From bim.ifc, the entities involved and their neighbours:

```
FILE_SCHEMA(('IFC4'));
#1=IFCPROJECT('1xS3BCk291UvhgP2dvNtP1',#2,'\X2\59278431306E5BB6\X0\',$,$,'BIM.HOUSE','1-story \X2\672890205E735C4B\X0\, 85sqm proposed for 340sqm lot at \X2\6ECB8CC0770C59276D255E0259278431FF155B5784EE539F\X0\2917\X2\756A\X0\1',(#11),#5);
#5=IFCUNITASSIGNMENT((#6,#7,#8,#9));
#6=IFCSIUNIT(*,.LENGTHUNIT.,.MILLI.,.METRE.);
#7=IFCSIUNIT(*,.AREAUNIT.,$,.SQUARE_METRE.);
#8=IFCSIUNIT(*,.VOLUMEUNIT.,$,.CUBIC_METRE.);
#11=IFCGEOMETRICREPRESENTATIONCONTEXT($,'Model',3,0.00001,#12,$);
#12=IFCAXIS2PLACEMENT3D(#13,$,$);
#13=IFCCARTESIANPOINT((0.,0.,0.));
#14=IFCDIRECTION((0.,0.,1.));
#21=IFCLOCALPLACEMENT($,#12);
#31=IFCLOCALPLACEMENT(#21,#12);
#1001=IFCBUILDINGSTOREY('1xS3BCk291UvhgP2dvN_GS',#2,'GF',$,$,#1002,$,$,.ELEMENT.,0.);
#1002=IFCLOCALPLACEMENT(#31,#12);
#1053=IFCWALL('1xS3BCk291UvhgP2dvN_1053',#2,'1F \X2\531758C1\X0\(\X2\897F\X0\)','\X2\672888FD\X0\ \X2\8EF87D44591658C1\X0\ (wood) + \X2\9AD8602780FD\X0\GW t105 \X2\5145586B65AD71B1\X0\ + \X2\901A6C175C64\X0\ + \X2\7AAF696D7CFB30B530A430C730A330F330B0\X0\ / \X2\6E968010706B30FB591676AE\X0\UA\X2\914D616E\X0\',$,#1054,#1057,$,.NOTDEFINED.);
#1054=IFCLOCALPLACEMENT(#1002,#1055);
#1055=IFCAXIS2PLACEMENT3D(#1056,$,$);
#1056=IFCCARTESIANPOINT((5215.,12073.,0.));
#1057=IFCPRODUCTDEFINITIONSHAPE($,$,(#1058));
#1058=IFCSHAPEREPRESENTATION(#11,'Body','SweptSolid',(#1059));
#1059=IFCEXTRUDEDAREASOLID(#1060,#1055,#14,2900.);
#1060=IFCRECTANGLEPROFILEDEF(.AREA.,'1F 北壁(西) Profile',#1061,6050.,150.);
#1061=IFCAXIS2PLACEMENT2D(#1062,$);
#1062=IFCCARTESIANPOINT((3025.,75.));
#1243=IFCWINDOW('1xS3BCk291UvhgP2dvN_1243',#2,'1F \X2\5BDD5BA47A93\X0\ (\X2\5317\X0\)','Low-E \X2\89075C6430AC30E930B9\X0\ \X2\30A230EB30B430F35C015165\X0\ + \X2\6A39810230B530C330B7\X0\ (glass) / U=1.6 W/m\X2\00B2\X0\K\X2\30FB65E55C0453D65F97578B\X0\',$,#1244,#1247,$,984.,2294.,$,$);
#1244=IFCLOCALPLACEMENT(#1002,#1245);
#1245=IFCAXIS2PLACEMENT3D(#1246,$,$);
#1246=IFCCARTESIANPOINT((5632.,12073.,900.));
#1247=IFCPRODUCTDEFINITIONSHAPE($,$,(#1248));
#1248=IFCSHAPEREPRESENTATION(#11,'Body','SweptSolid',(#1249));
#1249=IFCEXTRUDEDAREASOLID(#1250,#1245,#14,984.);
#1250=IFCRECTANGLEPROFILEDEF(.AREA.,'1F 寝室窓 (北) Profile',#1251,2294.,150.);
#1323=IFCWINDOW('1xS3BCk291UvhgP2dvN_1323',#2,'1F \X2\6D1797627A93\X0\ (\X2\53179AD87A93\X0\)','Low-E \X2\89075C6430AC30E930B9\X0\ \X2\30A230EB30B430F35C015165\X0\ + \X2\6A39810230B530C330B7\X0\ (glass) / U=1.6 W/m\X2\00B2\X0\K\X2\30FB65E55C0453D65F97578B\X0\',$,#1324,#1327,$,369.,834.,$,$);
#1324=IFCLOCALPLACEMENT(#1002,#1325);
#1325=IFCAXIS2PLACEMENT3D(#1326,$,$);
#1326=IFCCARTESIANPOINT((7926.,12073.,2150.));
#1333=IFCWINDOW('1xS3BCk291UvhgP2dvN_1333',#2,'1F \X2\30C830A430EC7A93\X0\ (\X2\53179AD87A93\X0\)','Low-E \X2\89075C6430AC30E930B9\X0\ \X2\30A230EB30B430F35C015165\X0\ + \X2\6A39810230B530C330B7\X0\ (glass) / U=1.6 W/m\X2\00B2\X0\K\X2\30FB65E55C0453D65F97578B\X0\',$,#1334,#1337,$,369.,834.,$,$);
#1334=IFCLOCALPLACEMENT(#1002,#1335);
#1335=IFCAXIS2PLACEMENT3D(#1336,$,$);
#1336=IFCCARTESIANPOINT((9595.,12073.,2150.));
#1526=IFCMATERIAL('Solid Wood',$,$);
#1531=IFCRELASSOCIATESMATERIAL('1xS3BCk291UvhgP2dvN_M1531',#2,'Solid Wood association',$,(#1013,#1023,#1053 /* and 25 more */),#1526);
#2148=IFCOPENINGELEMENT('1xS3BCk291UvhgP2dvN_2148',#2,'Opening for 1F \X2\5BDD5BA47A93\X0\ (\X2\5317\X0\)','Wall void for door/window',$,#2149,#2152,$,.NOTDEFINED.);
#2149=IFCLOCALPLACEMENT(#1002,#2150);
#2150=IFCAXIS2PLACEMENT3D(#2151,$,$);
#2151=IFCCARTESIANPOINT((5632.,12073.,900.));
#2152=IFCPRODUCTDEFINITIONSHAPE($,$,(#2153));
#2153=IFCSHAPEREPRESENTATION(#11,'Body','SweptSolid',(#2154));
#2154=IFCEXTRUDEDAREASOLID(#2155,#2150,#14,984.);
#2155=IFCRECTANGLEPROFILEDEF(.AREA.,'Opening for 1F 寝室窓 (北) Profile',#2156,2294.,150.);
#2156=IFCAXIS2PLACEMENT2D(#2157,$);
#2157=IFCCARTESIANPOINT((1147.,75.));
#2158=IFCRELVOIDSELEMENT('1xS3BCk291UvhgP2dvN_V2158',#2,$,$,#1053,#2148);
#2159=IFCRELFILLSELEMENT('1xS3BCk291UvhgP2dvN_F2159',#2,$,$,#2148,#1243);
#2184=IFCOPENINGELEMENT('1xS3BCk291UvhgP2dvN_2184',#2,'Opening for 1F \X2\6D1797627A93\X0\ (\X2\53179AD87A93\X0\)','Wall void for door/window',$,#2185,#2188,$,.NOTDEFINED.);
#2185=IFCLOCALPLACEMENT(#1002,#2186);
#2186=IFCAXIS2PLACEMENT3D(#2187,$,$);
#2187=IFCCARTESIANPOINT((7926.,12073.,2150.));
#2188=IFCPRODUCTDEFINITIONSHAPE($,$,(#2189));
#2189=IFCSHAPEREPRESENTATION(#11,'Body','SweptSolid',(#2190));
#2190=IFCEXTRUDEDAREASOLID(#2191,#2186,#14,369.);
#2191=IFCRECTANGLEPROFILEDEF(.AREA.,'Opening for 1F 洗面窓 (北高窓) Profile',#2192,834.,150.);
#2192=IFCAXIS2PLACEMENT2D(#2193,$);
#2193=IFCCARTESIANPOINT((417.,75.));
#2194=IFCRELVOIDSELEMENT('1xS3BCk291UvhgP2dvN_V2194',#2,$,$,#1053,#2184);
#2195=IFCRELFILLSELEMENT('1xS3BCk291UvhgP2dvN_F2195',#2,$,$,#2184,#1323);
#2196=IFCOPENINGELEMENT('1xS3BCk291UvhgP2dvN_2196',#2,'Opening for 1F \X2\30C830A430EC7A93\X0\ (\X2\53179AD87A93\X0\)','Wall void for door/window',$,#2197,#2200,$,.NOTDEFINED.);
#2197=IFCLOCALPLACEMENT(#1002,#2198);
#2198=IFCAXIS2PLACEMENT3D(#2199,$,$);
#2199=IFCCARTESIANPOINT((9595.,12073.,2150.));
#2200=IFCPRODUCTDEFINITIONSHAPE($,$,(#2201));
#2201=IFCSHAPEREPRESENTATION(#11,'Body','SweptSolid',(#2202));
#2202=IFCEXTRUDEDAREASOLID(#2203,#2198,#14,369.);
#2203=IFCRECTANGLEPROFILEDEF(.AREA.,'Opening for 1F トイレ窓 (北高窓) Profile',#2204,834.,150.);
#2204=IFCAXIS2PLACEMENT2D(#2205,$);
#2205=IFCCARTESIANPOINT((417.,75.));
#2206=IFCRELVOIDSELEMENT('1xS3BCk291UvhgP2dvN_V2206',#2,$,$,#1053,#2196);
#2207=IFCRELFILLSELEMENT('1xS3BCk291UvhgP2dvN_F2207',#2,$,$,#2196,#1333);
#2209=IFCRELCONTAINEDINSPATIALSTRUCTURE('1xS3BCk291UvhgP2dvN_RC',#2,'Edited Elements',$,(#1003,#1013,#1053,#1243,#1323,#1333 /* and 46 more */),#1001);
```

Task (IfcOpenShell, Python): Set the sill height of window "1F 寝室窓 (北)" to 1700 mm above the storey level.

```python
import numpy as np
import ifcopenshell
import ifcopenshell.api.geometry
import ifcopenshell.geom
import ifcopenshell.util.element
import ifcopenshell.util.placement
import ifcopenshell.util.shape
import ifcopenshell.util.unit

model = ifcopenshell.open("bim.ifc")
unit_scale = ifcopenshell.util.unit.calculate_unit_scale(model)

window = model.by_id(1243)
opening = window.FillsVoids[0].RelatingOpeningElement
storey = ifcopenshell.util.element.get_container(window, ifc_class="IfcBuildingStorey")
level = ifcopenshell.util.placement.get_local_placement(storey.ObjectPlacement)[2, 3]

# The opening's origin need not be at the sill, so measure its lowest point.
shape = ifcopenshell.geom.create_shape(ifcopenshell.geom.settings(), opening)
bottom = ifcopenshell.util.shape.get_shape_bottom_elevation(shape, shape.geometry) / unit_scale
dz = level + 1700.0 - bottom

shift = np.array([0.0, 0.0, dz])
# The window is not placed relative to its opening, so move both.
for product in (opening, window):
    matrix = ifcopenshell.util.placement.get_local_placement(product.ObjectPlacement)
    matrix[:3, 3] += shift
    ifcopenshell.api.geometry.edit_object_placement(model, product=product, matrix=matrix, is_si=False)

print(f"moved by {dz * unit_scale:+.3f} m")

model.write("bim_updated.ifc")
```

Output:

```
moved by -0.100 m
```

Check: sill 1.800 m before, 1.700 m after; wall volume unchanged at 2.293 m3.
